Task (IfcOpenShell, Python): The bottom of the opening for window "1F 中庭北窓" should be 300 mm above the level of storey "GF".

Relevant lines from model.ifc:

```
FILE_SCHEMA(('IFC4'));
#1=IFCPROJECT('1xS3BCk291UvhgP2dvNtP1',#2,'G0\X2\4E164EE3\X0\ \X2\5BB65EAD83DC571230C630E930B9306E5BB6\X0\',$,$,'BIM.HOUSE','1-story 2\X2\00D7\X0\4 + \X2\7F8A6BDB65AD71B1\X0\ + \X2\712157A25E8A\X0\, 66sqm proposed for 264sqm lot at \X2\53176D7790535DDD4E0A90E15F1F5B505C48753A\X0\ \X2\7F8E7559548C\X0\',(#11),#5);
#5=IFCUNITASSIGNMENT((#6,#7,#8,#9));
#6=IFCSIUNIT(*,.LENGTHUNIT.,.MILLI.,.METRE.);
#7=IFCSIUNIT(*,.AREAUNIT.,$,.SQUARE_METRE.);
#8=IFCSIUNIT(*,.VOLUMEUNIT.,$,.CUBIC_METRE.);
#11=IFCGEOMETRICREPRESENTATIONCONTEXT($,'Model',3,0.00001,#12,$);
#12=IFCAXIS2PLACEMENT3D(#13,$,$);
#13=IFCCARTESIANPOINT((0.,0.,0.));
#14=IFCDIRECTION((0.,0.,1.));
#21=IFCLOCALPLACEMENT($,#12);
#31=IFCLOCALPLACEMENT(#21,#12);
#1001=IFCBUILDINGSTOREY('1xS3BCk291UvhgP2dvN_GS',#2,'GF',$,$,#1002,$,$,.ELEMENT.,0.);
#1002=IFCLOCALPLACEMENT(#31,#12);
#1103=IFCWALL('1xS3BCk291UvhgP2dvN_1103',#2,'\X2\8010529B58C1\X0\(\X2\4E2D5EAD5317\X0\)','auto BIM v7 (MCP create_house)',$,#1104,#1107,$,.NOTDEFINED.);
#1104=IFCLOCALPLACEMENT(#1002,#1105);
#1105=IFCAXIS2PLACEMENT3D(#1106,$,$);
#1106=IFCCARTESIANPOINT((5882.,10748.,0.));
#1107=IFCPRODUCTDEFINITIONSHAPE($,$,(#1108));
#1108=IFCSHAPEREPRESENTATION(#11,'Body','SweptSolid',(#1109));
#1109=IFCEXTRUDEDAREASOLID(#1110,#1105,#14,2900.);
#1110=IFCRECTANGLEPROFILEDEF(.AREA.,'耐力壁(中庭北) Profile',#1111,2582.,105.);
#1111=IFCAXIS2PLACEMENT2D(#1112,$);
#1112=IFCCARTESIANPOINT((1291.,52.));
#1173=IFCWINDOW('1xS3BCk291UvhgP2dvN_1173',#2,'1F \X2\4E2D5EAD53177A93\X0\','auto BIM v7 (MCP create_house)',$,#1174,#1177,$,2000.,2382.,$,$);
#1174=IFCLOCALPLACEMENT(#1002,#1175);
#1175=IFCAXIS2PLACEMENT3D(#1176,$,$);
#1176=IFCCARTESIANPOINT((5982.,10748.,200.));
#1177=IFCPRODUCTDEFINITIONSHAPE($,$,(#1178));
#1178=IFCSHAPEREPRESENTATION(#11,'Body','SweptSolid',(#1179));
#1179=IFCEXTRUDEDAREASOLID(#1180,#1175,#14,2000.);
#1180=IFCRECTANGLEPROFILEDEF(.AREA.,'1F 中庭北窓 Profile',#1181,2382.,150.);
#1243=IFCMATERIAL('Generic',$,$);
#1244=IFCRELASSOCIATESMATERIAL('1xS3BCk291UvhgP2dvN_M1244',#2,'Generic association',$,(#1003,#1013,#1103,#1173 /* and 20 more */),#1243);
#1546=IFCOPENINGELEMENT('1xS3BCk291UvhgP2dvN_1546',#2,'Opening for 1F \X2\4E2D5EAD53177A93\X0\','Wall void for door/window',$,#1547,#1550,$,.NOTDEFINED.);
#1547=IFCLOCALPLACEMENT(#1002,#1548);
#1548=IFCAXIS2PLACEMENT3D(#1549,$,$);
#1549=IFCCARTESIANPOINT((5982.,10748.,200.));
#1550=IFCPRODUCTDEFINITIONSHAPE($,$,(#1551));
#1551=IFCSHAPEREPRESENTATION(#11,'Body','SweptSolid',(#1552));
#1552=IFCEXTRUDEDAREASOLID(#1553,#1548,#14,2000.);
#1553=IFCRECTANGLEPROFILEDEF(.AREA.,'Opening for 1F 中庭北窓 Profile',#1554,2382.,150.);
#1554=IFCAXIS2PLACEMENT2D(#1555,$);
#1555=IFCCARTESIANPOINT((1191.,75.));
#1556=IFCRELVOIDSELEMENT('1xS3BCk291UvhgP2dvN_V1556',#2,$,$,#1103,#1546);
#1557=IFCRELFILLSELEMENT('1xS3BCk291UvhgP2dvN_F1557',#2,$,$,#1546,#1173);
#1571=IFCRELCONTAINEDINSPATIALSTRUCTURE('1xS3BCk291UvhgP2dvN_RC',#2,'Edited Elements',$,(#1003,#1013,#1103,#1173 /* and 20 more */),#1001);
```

```python
import numpy as np
import ifcopenshell
import ifcopenshell.api.geometry
import ifcopenshell.geom
import ifcopenshell.util.element
import ifcopenshell.util.placement
import ifcopenshell.util.shape
import ifcopenshell.util.unit

model = ifcopenshell.open("model.ifc")
unit_scale = ifcopenshell.util.unit.calculate_unit_scale(model)

window = model.by_guid("1xS3BCk291UvhgP2dvN_1173")
opening = window.FillsVoids[0].RelatingOpeningElement
storey = ifcopenshell.util.element.get_container(window, ifc_class="IfcBuildingStorey")
level = ifcopenshell.util.placement.get_local_placement(storey.ObjectPlacement)[2, 3]

# The opening's origin need not be at the sill, so measure its lowest point.
shape = ifcopenshell.geom.create_shape(ifcopenshell.geom.settings(), opening)
bottom = ifcopenshell.util.shape.get_shape_bottom_elevation(shape, shape.geometry) / unit_scale
dz = level + 0.3 / unit_scale - bottom

shift = np.array([0.0, 0.0, dz])
# The window is not placed relative to its opening, so move both.
for product in (opening, window):
    matrix = ifcopenshell.util.placement.get_local_placement(product.ObjectPlacement)
    matrix[:3, 3] += shift
    ifcopenshell.api.geometry.edit_object_placement(model, product=product, matrix=matrix, is_si=False)

print(f"moved by {dz * unit_scale:+.3f} m")

model.write("model_v2.ifc")
```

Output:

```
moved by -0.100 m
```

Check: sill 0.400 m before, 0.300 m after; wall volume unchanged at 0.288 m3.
